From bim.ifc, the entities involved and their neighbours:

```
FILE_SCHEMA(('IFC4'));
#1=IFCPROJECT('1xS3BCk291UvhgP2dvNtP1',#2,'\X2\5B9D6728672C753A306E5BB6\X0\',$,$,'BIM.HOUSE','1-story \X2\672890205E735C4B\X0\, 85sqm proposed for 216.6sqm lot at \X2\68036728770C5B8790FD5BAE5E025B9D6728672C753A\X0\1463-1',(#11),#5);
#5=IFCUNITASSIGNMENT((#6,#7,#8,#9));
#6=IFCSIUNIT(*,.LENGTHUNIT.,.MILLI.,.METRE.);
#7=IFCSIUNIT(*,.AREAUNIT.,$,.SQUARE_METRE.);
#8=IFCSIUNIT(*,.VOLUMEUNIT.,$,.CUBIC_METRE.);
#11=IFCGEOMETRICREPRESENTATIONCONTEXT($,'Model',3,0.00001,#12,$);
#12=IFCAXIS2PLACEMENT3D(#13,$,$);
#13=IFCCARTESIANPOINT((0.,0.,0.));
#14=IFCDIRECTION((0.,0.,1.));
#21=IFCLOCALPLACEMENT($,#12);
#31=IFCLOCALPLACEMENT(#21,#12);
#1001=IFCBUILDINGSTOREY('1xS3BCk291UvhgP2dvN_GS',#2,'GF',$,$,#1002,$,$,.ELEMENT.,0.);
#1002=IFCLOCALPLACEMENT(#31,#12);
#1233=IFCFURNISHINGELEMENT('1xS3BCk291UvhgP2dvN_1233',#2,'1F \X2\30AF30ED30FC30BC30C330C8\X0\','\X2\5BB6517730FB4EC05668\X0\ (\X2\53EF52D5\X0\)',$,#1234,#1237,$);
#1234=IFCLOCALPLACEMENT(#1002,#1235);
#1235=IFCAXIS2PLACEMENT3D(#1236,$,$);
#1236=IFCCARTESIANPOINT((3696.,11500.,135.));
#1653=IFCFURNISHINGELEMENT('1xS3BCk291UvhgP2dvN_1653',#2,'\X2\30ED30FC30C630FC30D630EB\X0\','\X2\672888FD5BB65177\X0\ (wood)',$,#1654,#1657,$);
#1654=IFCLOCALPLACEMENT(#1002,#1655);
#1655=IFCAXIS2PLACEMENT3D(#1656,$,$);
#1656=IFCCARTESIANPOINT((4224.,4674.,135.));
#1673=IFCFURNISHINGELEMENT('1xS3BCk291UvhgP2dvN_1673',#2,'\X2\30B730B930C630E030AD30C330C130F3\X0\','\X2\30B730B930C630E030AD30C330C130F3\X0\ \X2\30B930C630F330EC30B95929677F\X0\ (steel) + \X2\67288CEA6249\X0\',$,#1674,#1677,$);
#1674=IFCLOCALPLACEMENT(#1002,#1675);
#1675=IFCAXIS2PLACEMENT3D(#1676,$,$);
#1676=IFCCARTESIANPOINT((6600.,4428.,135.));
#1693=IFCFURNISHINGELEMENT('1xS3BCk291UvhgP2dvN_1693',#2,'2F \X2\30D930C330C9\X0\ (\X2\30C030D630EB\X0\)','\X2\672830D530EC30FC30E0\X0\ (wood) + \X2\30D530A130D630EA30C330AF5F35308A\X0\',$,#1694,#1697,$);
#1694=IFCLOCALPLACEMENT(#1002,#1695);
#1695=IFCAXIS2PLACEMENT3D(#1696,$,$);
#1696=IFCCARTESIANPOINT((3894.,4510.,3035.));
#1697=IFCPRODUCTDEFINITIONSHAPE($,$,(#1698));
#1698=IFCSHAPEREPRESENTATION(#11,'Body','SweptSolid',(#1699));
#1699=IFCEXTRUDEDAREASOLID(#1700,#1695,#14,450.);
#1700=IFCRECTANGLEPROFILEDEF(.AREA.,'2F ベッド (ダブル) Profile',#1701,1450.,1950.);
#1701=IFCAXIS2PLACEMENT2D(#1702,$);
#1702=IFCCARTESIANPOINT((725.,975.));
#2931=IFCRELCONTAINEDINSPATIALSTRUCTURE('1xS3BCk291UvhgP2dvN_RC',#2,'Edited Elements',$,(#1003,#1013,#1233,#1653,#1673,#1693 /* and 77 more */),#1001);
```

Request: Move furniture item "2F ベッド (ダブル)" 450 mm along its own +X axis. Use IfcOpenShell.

```python
import ifcopenshell
import ifcopenshell.api.geometry
import ifcopenshell.util.placement
import ifcopenshell.util.unit

model = ifcopenshell.open("bim.ifc")
unit_scale = ifcopenshell.util.unit.calculate_unit_scale(model)

item = model.by_guid("1xS3BCk291UvhgP2dvN_1693")
matrix = ifcopenshell.util.placement.get_local_placement(item.ObjectPlacement)
matrix[:3, 3] += matrix[:3, 0] * 0.45 / unit_scale
ifcopenshell.api.geometry.edit_object_placement(model, product=item, matrix=matrix, is_si=False)

print(ifcopenshell.util.placement.get_local_placement(item.ObjectPlacement).round(3) + 0.0)

model.write("bim-out.ifc")
```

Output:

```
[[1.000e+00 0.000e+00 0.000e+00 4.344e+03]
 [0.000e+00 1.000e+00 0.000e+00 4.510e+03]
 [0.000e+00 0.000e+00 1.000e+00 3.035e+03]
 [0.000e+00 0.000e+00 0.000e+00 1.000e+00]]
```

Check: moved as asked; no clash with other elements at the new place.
